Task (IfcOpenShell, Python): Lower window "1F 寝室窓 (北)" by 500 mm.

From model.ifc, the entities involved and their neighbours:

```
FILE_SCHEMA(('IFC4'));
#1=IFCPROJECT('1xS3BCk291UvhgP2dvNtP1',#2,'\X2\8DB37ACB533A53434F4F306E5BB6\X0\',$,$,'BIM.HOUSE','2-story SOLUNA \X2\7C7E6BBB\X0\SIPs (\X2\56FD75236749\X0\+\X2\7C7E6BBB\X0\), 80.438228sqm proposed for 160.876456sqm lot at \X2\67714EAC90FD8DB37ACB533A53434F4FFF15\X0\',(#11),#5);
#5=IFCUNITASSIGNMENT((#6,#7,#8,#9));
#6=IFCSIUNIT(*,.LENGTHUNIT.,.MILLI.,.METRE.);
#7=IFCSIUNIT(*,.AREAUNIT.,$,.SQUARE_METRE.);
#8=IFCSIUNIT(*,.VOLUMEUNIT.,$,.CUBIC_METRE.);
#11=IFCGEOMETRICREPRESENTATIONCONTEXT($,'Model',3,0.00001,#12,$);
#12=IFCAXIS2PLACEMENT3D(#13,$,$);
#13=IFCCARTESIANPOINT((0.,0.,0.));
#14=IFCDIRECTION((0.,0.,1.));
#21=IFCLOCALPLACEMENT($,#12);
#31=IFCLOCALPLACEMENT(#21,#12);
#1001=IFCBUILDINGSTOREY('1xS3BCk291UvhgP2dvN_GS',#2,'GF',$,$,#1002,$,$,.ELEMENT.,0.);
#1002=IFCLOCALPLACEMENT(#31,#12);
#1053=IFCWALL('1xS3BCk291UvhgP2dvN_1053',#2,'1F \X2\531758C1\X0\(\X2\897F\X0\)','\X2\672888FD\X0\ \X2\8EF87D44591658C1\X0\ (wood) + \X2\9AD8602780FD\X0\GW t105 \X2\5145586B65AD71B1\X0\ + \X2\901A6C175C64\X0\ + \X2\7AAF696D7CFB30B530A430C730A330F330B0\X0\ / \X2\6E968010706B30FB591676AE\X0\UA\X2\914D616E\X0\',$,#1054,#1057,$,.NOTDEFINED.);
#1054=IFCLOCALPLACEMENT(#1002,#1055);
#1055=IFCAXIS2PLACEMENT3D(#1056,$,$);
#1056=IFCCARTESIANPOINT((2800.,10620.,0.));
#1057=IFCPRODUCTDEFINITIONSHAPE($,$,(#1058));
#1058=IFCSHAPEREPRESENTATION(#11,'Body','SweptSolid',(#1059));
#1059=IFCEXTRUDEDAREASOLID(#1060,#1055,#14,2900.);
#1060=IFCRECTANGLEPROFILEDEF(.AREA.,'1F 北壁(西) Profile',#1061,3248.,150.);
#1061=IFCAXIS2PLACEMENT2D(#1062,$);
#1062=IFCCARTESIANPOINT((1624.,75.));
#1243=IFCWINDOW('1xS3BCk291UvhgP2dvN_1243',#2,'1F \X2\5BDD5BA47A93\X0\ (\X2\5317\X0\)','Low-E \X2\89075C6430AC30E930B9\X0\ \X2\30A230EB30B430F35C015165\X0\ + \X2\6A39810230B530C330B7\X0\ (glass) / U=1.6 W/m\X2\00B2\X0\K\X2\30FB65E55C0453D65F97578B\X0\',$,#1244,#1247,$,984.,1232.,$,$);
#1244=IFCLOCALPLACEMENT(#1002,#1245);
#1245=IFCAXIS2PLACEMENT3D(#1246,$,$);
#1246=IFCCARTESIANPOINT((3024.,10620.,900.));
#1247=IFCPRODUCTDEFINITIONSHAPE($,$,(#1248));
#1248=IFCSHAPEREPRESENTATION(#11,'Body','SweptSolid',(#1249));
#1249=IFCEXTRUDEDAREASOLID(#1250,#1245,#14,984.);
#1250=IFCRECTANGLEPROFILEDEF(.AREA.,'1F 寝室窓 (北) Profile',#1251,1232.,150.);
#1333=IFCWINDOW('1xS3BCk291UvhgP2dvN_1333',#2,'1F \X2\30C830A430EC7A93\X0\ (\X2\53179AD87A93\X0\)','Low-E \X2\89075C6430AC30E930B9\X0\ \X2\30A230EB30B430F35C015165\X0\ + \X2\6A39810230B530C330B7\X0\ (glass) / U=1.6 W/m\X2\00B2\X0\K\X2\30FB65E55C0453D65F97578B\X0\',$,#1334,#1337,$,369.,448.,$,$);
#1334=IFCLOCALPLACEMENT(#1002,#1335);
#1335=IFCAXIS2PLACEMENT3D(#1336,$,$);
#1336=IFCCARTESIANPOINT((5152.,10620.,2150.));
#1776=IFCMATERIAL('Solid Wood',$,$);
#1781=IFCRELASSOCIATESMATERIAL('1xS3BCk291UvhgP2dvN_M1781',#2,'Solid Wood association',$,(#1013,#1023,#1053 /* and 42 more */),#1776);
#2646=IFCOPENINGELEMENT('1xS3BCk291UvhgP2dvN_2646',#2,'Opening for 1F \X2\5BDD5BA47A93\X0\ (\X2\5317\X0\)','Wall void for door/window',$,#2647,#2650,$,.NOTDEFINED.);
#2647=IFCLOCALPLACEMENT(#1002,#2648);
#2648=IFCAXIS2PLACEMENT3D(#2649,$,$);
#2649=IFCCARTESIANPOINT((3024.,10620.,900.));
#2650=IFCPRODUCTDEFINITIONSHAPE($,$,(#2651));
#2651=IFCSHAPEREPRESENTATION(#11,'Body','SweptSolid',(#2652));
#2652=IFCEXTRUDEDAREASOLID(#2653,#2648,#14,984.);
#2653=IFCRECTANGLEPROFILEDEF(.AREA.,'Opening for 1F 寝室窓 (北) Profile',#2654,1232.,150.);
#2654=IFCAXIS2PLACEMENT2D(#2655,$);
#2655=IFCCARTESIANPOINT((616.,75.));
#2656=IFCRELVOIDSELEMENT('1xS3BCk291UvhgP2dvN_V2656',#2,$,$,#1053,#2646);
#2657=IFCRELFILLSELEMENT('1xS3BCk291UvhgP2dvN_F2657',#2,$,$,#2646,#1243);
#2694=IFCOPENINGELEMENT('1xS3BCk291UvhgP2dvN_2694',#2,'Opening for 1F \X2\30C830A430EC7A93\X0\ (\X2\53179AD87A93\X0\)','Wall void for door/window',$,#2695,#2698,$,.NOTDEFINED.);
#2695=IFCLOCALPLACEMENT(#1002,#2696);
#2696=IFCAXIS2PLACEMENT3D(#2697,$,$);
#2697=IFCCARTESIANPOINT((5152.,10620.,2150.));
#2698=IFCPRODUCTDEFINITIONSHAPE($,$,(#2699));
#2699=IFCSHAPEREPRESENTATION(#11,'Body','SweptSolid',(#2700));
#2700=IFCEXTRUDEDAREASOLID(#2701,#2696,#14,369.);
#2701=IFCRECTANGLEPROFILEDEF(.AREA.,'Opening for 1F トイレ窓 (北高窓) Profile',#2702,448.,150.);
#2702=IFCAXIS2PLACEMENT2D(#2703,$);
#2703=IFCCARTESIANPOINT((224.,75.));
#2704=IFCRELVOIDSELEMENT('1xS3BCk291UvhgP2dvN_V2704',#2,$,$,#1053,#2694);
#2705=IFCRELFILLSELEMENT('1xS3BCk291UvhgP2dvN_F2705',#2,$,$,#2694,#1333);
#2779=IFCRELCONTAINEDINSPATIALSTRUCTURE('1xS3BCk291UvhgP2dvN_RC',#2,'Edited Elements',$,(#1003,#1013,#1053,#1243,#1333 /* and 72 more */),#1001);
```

```python
import numpy as np
import ifcopenshell
import ifcopenshell.api.geometry
import ifcopenshell.util.placement
import ifcopenshell.util.unit

model = ifcopenshell.open("model.ifc")
unit_scale = ifcopenshell.util.unit.calculate_unit_scale(model)

window = model.by_guid("1xS3BCk291UvhgP2dvN_1243")
opening = window.FillsVoids[0].RelatingOpeningElement
dz = -500.0

shift = np.array([0.0, 0.0, dz])
# The window is not placed relative to its opening, so move both.
for product in (opening, window):
    matrix = ifcopenshell.util.placement.get_local_placement(product.ObjectPlacement)
    matrix[:3, 3] += shift
    ifcopenshell.api.geometry.edit_object_placement(model, product=product, matrix=matrix, is_si=False)

print(f"moved by {dz * unit_scale:+.3f} m")

model.write("model_updated.ifc")
```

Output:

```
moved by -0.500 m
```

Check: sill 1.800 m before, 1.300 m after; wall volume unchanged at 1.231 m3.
